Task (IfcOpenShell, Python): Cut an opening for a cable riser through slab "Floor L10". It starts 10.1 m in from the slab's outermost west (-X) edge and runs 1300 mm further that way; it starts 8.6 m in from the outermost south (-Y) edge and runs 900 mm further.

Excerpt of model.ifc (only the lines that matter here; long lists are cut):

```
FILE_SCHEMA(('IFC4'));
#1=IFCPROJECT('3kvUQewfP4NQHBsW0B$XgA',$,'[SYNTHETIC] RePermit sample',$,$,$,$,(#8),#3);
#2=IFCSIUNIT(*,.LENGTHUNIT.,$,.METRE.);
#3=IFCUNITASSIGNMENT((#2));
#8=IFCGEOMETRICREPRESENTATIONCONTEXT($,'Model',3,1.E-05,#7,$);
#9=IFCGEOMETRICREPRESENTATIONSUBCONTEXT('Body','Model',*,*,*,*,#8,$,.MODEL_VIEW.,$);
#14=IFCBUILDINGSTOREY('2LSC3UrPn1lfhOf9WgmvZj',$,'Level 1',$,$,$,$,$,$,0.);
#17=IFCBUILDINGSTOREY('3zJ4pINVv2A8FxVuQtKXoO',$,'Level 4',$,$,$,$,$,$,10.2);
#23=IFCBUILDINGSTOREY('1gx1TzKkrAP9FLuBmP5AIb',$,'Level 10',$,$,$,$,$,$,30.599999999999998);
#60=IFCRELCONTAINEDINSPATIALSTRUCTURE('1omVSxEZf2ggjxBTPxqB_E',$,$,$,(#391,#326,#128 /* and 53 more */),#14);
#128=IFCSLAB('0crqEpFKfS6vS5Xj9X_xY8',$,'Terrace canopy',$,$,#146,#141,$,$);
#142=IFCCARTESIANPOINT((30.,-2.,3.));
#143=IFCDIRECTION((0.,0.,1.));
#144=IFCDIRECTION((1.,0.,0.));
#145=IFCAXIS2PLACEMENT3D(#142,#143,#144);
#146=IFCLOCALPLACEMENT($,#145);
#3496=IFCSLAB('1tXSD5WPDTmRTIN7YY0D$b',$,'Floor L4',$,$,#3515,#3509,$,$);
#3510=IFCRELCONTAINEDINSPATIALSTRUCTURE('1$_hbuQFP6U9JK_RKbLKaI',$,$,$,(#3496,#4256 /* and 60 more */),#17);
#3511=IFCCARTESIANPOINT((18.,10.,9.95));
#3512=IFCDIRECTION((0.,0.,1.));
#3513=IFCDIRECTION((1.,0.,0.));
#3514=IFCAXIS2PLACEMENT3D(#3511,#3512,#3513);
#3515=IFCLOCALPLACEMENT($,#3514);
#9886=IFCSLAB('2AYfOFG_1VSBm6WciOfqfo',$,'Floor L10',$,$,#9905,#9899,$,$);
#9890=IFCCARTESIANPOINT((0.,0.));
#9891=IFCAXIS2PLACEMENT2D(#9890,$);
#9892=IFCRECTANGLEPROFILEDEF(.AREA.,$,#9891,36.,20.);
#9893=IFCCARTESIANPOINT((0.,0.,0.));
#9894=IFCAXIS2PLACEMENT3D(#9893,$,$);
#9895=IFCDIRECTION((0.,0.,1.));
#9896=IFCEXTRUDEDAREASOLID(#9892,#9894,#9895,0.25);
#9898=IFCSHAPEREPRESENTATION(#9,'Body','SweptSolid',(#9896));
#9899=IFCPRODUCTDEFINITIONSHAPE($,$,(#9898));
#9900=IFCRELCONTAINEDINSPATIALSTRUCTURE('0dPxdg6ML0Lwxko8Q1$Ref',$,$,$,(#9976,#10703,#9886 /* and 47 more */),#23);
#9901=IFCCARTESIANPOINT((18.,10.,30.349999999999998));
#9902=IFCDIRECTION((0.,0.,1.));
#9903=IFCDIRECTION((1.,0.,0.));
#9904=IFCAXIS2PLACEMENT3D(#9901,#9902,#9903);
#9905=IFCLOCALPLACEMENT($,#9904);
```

```python
import numpy as np
import ifcopenshell
import ifcopenshell.api.feature
import ifcopenshell.api.geometry
import ifcopenshell.api.root
import ifcopenshell.geom
import ifcopenshell.util.placement
import ifcopenshell.util.representation
import ifcopenshell.util.shape
import ifcopenshell.util.unit

model = ifcopenshell.open("model.ifc")
unit_scale = ifcopenshell.util.unit.calculate_unit_scale(model)
settings = ifcopenshell.geom.settings()


def volume(element):
    """Net volume in cubic metres, openings subtracted."""
    shape = ifcopenshell.geom.create_shape(settings, element)
    return ifcopenshell.util.shape.get_volume(shape.geometry)


slab = model.by_guid("2AYfOFG_1VSBm6WciOfqfo")
before = volume(slab)

# Extent in the slab's own axes, in metres. The edges named are its -X and -Y sides.
slab_shape = ifcopenshell.geom.create_shape(settings, slab)
vertices = ifcopenshell.util.shape.get_vertices(slab_shape.geometry)
x_min, y_min, bottom = vertices.min(axis=0)
top = vertices[:, 2].max()

opening = ifcopenshell.api.root.create_entity(model, ifc_class="IfcOpeningElement", name="Cable riser opening", predefined_type="OPENING")
context = ifcopenshell.util.representation.get_context(model, "Model", "Body", "MODEL_VIEW")
width, depth = 1.3, 0.9
outline = [(0.0, 0.0), (width, 0.0), (width, depth), (0.0, depth), (0.0, 0.0)]
# Overshoot both faces by 50 mm so the cut is clean.
shape = ifcopenshell.api.geometry.add_slab_representation(
    model, context=context, depth=top - bottom + 0.1, polyline=outline
)
ifcopenshell.api.geometry.assign_representation(model, product=opening, representation=shape)

matrix = ifcopenshell.util.placement.get_local_placement(slab.ObjectPlacement)
matrix[:, 3] = matrix @ np.append(np.array([x_min + 10.1, y_min + 8.6, bottom - 0.05]) / unit_scale, 1.0)
ifcopenshell.api.geometry.edit_object_placement(model, product=opening, matrix=matrix, is_si=False)
ifcopenshell.api.feature.add_feature(model, feature=opening, element=slab)

after = volume(slab)

print(f"slab volume {before:.3f} -> {after:.3f} m3")

model.write("model_edited.ifc")
```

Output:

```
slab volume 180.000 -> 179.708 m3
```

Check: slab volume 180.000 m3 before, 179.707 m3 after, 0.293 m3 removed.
